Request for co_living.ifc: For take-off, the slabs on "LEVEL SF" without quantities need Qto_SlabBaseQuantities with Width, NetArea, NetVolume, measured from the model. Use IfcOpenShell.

First a look at what the model holds.

```python
import ifcopenshell
import ifcopenshell.util.element
import ifcopenshell.util.unit

model = ifcopenshell.open("co_living.ifc")
print(model.schema)
for unit_type in ("LENGTHUNIT", "AREAUNIT", "VOLUMEUNIT"):
    print(unit_type, ifcopenshell.util.unit.calculate_unit_scale(model, unit_type))
storey = next(s for s in model.by_type("IfcBuildingStorey") if s.Name == "LEVEL SF")
slabs = [e for e in ifcopenshell.util.element.get_decomposition(storey) if e.is_a("IfcSlab")]
for e in sorted(slabs, key=lambda e: e.id()):
    print(e.id(), e.is_a(), e.Name, list(ifcopenshell.util.element.get_psets(e, qtos_only=True)), sep=" | ")
```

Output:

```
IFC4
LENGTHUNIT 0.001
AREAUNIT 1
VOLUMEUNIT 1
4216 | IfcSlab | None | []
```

```python
import ifcopenshell
import ifcopenshell.api.pset
import ifcopenshell.geom
import ifcopenshell.util.element
import ifcopenshell.util.shape
import ifcopenshell.util.unit

model = ifcopenshell.open("co_living.ifc")
unit_scale = ifcopenshell.util.unit.calculate_unit_scale(model)
area_scale = ifcopenshell.util.unit.calculate_unit_scale(model, "AREAUNIT")
volume_scale = ifcopenshell.util.unit.calculate_unit_scale(model, "VOLUMEUNIT")
settings = ifcopenshell.geom.settings()

storey = next(s for s in model.by_type("IfcBuildingStorey") if s.Name == "LEVEL SF")
slabs = [e for e in ifcopenshell.util.element.get_decomposition(storey) if e.is_a("IfcSlab")]

for e in sorted(slabs, key=lambda e: e.id()):
    if ifcopenshell.util.element.get_psets(e, qtos_only=True, should_inherit=False):
        continue
    # Geometry comes back in metres, in the element's own axes.
    shape = ifcopenshell.geom.create_shape(settings, e)
    values = {
        "Width": ifcopenshell.util.shape.get_z(shape.geometry) / unit_scale,
        "NetArea": ifcopenshell.util.shape.get_footprint_area(shape.geometry) / area_scale,
        "NetVolume": ifcopenshell.util.shape.get_volume(shape.geometry) / volume_scale,
    }
    qto = ifcopenshell.api.pset.add_qto(model, product=e, name="Qto_SlabBaseQuantities")
    ifcopenshell.api.pset.edit_qto(model, qto=qto, properties=values)
    print(e.id(), {k: round(v, 3) for k, v in values.items()})

model.write("co_living_updated.ifc")
```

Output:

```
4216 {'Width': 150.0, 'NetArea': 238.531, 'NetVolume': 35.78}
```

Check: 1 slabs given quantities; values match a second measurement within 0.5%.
